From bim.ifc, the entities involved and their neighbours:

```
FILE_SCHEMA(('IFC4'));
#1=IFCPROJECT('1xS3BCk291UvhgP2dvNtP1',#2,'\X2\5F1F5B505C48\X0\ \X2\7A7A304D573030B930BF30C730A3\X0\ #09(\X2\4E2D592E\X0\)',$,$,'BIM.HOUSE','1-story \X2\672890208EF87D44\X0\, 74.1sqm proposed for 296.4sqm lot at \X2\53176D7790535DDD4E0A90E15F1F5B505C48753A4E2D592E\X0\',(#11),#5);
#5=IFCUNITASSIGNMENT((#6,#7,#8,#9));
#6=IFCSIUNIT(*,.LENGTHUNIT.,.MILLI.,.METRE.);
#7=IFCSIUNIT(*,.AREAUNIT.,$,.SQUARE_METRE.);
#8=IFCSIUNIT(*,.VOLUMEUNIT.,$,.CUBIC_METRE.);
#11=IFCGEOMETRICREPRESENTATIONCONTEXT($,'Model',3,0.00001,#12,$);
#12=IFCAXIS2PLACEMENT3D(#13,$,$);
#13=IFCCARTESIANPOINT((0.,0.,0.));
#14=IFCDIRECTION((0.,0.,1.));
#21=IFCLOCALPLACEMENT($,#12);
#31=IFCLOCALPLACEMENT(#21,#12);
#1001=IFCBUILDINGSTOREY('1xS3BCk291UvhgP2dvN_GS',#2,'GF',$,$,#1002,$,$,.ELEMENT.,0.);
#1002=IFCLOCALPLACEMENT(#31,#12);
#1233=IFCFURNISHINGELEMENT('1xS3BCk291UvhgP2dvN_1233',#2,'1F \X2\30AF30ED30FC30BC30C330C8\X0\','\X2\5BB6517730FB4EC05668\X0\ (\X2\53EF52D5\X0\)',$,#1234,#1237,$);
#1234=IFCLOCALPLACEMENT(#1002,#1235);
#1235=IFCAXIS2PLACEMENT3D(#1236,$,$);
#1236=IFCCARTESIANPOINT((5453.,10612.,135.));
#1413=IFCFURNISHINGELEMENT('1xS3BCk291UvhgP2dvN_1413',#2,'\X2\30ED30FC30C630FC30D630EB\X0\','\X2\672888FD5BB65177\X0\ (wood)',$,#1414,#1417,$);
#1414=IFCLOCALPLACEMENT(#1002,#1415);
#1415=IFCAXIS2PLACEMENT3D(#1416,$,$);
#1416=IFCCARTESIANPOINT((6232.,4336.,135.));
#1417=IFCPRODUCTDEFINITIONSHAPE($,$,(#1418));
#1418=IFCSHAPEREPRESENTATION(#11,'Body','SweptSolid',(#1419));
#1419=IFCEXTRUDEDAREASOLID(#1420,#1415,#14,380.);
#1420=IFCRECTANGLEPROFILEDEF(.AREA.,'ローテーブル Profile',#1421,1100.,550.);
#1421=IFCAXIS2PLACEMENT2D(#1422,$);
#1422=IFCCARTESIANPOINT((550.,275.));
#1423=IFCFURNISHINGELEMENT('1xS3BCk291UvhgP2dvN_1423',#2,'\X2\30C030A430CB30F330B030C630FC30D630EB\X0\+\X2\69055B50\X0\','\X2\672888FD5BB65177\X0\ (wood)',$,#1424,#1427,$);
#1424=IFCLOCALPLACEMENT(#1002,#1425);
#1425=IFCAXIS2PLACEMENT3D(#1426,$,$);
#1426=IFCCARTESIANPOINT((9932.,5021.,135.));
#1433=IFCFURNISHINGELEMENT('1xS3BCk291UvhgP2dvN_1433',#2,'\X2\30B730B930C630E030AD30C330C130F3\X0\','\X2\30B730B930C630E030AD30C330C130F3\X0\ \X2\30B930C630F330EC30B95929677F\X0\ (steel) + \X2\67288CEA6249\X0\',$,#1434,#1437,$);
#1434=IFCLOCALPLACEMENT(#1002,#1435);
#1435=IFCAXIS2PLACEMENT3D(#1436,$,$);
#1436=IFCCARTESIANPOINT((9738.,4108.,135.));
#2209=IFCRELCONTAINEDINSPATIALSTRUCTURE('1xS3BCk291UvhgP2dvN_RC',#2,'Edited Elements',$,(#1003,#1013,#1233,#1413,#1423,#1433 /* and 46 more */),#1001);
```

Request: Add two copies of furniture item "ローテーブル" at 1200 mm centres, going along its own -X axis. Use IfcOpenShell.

```python
import ifcopenshell
import ifcopenshell.api.geometry
import ifcopenshell.api.root
import ifcopenshell.util.element
import ifcopenshell.util.placement

model = ifcopenshell.open("bim.ifc")


def reuse_history(source, copy):
    """copy_class also copies each property set's owner history, people and application; keep the originals."""
    for rel in copy.IsDefinedBy:
        if rel.is_a("IfcRelDefinesByProperties") and (history := rel.RelatingPropertyDefinition.OwnerHistory):
            rel.RelatingPropertyDefinition.OwnerHistory = source.OwnerHistory
            ifcopenshell.util.element.remove_deep2(model, history)


source = model.by_id(1413)
base = ifcopenshell.util.placement.get_local_placement(source.ObjectPlacement)
step = -base[:3, 0] * 1200.0

for i in range(1, 3):
    copy = ifcopenshell.api.root.copy_class(model, product=source)
    copy.Representation = ifcopenshell.util.element.copy_deep(
        model, source.Representation, exclude=["IfcGeometricRepresentationContext", "IfcRepresentationMap"]
    )
    reuse_history(source, copy)
    matrix = base.copy()
    matrix[:3, 3] += i * step
    print("added at", matrix[:3, 3].round(3) + 0.0)
    ifcopenshell.api.geometry.edit_object_placement(model, product=copy, matrix=matrix, is_si=False)

model.write("bim_updated.ifc")
```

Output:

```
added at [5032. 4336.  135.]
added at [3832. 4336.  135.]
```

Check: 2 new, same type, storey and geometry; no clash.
